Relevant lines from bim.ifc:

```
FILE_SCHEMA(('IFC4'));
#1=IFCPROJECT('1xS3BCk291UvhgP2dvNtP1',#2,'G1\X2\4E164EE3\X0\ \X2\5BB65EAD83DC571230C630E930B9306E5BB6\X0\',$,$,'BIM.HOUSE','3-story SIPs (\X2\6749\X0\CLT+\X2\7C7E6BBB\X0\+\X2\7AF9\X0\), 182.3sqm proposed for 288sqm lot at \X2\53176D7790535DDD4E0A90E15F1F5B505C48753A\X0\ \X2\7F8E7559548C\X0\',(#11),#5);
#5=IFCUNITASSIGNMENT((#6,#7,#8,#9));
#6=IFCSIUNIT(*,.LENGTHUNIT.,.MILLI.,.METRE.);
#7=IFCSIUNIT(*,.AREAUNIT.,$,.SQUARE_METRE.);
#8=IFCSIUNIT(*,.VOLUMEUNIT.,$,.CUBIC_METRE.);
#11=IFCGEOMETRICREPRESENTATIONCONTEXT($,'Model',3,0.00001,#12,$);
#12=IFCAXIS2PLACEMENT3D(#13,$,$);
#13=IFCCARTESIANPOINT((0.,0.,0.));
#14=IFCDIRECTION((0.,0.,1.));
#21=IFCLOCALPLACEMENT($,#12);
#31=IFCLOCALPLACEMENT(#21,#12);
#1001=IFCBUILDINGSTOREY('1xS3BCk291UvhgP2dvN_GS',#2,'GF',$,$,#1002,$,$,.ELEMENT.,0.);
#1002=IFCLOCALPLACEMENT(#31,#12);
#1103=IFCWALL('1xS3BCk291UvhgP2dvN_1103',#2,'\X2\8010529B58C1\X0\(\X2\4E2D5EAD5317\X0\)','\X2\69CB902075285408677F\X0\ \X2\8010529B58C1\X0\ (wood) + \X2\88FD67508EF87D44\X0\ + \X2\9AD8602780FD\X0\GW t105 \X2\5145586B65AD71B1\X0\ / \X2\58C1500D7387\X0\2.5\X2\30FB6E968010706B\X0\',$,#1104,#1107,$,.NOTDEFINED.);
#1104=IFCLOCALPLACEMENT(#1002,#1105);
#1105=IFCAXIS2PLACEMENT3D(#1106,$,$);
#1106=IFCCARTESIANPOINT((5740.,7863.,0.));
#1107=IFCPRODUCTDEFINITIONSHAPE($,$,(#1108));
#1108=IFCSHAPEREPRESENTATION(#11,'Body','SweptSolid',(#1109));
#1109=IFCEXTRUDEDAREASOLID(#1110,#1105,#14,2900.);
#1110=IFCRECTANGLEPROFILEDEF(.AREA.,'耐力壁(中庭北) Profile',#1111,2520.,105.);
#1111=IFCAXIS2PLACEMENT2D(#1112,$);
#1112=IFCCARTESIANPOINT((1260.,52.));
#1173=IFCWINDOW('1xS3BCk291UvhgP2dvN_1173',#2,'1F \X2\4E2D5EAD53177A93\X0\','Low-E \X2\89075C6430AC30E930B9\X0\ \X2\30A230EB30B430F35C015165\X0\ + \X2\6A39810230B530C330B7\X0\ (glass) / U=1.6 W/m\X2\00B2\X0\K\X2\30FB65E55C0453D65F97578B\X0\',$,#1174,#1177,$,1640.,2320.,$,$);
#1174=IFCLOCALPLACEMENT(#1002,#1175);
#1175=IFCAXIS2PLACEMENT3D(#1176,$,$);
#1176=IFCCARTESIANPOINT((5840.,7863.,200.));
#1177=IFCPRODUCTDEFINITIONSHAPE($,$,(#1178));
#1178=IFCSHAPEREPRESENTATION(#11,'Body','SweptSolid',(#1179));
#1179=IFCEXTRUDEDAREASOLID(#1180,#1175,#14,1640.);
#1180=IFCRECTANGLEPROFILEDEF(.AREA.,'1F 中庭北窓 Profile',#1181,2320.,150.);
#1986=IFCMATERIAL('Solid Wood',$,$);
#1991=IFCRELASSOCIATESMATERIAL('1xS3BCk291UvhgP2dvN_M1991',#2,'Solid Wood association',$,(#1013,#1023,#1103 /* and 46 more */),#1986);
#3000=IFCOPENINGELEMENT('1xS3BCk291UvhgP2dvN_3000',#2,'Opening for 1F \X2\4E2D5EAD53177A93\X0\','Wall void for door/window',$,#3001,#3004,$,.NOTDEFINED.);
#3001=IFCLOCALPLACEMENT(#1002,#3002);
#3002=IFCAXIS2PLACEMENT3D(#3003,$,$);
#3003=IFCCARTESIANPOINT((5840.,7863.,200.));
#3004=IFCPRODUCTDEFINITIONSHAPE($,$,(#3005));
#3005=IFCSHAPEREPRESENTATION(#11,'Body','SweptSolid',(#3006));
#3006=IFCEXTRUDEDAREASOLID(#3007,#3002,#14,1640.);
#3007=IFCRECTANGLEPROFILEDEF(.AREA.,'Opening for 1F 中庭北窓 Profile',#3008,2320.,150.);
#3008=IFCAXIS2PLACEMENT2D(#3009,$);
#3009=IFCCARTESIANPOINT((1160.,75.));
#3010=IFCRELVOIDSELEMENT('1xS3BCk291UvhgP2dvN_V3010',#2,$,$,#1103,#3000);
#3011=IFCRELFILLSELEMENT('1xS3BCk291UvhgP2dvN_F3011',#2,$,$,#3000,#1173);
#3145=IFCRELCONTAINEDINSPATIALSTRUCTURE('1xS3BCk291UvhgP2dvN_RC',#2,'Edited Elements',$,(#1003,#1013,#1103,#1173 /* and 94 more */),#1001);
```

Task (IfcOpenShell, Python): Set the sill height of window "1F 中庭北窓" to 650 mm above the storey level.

```python
import numpy as np
import ifcopenshell
import ifcopenshell.api.geometry
import ifcopenshell.geom
import ifcopenshell.util.element
import ifcopenshell.util.placement
import ifcopenshell.util.shape
import ifcopenshell.util.unit

model = ifcopenshell.open("bim.ifc")
unit_scale = ifcopenshell.util.unit.calculate_unit_scale(model)

window = model.by_guid("1xS3BCk291UvhgP2dvN_1173")
opening = window.FillsVoids[0].RelatingOpeningElement
storey = ifcopenshell.util.element.get_container(window, ifc_class="IfcBuildingStorey")
level = ifcopenshell.util.placement.get_local_placement(storey.ObjectPlacement)[2, 3]

# The opening's origin need not be at the sill, so measure its lowest point.
shape = ifcopenshell.geom.create_shape(ifcopenshell.geom.settings(), opening)
bottom = ifcopenshell.util.shape.get_shape_bottom_elevation(shape, shape.geometry) / unit_scale
dz = level + 650.0 - bottom

shift = np.array([0.0, 0.0, dz])
# The window is not placed relative to its opening, so move both.
for product in (opening, window):
    matrix = ifcopenshell.util.placement.get_local_placement(product.ObjectPlacement)
    matrix[:3, 3] += shift
    ifcopenshell.api.geometry.edit_object_placement(model, product=product, matrix=matrix, is_si=False)

print(f"moved by {dz * unit_scale:+.3f} m")

model.write("bim_edited.ifc")
```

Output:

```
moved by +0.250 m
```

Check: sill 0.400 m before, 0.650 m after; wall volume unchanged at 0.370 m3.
